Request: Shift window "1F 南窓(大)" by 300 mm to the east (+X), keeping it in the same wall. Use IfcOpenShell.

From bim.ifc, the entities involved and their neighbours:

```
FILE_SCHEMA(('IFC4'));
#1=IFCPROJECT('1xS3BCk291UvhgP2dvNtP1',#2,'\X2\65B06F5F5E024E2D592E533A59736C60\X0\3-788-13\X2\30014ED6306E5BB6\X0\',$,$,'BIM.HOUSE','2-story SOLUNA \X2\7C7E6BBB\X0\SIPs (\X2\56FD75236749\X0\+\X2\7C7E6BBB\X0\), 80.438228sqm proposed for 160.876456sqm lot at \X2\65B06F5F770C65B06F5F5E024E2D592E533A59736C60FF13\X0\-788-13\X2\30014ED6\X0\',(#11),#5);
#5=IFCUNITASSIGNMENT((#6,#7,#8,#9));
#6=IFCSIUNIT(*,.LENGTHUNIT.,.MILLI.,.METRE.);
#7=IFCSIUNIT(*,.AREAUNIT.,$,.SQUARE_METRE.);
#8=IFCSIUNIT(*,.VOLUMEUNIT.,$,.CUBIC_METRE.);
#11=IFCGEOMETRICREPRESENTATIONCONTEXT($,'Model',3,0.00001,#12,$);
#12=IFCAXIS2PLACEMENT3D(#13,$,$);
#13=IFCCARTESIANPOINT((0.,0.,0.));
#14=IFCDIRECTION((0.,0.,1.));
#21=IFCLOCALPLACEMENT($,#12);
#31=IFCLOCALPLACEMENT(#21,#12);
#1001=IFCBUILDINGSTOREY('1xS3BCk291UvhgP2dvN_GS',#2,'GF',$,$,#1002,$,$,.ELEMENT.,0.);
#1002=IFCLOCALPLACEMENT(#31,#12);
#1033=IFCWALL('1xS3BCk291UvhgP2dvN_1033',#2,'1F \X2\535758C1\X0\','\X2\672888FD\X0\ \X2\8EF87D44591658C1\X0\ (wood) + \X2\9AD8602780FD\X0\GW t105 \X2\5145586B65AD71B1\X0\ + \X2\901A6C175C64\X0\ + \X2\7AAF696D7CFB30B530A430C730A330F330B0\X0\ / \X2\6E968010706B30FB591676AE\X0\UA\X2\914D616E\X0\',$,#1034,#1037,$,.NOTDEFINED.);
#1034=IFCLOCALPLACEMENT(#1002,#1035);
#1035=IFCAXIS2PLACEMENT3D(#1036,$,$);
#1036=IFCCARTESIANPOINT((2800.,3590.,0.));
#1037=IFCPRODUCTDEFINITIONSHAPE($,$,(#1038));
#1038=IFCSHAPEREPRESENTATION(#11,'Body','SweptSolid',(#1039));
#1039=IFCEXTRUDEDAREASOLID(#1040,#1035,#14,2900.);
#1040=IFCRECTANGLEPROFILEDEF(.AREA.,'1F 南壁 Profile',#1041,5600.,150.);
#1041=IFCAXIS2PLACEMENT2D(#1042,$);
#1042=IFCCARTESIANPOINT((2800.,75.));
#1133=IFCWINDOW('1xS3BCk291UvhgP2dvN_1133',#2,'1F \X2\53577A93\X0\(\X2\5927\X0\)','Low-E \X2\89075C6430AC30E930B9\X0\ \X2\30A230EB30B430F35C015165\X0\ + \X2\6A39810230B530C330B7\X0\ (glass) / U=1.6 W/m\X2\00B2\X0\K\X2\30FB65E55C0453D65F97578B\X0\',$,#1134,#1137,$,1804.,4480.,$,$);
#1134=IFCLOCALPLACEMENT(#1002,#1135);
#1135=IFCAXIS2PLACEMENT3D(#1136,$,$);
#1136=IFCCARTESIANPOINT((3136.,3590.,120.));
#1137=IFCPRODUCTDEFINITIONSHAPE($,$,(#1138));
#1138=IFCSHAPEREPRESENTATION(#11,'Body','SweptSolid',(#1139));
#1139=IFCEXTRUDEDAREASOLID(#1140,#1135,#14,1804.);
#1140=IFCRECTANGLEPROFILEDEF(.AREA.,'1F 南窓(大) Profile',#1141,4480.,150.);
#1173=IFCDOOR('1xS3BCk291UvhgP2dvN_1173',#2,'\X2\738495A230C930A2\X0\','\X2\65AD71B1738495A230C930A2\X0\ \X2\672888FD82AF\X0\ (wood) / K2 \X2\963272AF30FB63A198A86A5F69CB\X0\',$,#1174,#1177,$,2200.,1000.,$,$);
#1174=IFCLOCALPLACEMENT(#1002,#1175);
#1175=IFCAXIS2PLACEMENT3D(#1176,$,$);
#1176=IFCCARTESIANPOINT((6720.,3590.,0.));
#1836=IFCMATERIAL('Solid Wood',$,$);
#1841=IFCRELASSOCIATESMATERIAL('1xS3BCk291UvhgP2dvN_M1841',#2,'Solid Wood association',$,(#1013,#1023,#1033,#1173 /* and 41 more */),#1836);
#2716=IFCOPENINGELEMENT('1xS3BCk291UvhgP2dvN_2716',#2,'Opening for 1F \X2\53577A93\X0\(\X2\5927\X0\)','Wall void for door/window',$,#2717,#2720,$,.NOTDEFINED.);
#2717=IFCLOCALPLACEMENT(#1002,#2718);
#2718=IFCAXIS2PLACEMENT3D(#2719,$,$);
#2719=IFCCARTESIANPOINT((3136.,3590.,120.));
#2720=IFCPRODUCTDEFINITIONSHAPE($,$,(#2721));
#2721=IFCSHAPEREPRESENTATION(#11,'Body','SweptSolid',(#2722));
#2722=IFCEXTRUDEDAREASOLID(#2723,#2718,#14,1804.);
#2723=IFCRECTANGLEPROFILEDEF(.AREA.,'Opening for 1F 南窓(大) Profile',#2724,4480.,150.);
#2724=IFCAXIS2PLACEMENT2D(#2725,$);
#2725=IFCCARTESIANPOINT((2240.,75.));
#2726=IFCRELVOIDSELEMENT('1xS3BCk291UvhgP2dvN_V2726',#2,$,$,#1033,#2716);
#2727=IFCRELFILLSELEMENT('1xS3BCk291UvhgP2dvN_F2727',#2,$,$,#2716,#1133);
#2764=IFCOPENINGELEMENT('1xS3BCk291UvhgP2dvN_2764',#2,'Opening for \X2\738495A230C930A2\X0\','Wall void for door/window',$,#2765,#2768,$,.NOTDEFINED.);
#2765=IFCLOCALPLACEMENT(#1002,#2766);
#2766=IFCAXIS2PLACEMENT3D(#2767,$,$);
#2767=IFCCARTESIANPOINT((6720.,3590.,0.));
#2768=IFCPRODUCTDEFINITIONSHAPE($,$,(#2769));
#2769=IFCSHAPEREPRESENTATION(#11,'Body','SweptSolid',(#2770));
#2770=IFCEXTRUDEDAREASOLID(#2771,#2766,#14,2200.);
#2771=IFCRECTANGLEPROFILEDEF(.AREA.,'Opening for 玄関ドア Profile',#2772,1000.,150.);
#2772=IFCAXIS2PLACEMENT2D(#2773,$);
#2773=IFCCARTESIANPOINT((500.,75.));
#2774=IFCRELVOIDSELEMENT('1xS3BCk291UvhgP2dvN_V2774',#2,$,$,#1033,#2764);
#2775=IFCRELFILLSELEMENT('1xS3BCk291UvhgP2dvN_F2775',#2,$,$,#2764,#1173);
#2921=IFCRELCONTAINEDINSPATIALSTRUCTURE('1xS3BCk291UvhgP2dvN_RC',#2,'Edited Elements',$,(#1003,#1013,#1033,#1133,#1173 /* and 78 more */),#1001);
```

```python
import ifcopenshell
import ifcopenshell.api.geometry
import ifcopenshell.util.placement
import ifcopenshell.util.unit

model = ifcopenshell.open("bim.ifc")
unit_scale = ifcopenshell.util.unit.calculate_unit_scale(model)

window = model.by_guid("1xS3BCk291UvhgP2dvN_1133")
opening = window.FillsVoids[0].RelatingOpeningElement
wall = opening.VoidsElements[0].RelatingBuildingElement

wall_matrix = ifcopenshell.util.placement.get_local_placement(wall.ObjectPlacement)
shift = wall_matrix[:3, 0] * 0.3 / unit_scale
before = ifcopenshell.util.placement.get_local_placement(window.ObjectPlacement)[:3, 3].copy()

# The window is not placed relative to its opening, so move both.
for product in (opening, window):
    matrix = ifcopenshell.util.placement.get_local_placement(product.ObjectPlacement)
    matrix[:3, 3] += shift
    ifcopenshell.api.geometry.edit_object_placement(model, product=product, matrix=matrix, is_si=False)

after = ifcopenshell.util.placement.get_local_placement(window.ObjectPlacement)[:3, 3]
print("window moved by", (after - before).round(3) + 0.0)

model.write("bim_edited.ifc")
```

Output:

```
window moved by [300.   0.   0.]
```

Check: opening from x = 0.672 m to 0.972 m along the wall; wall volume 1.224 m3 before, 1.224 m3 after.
